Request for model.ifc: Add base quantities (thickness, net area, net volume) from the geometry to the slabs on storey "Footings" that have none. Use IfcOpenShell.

First a look at what the model holds.

```python
import ifcopenshell
import ifcopenshell.util.element
import ifcopenshell.util.unit

model = ifcopenshell.open("model.ifc")
print(model.schema)
for unit_type in ("LENGTHUNIT", "AREAUNIT", "VOLUMEUNIT"):
    print(unit_type, ifcopenshell.util.unit.calculate_unit_scale(model, unit_type))
storey = next(s for s in model.by_type("IfcBuildingStorey") if s.Name == "Footings")
slabs = [e for e in ifcopenshell.util.element.get_decomposition(storey) if e.is_a("IfcSlab")]
for e in sorted(slabs, key=lambda e: e.id()):
    print(e.id(), e.is_a(), e.Name, list(ifcopenshell.util.element.get_psets(e, qtos_only=True)), sep=" | ")
```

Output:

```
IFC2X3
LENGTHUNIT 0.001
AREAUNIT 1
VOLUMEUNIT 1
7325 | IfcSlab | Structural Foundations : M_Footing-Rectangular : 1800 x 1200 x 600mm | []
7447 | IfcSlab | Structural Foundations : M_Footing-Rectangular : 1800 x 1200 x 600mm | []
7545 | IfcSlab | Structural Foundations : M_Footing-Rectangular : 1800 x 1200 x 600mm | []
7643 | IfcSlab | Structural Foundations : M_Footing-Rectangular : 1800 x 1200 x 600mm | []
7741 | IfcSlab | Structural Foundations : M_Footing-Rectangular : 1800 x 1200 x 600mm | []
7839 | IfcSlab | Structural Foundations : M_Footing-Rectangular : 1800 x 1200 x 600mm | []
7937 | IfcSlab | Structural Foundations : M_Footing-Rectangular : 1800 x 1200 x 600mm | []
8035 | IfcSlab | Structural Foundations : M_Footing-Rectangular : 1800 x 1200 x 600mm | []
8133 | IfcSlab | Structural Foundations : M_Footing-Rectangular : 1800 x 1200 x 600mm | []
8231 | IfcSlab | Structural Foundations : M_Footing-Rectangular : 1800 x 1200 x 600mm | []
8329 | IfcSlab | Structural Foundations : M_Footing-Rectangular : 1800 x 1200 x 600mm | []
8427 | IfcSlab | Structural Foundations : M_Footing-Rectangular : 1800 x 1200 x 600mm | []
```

```python
import ifcopenshell
import ifcopenshell.api.pset
import ifcopenshell.geom
import ifcopenshell.util.element
import ifcopenshell.util.shape
import ifcopenshell.util.unit

model = ifcopenshell.open("model.ifc")
unit_scale = ifcopenshell.util.unit.calculate_unit_scale(model)
area_scale = ifcopenshell.util.unit.calculate_unit_scale(model, "AREAUNIT")
volume_scale = ifcopenshell.util.unit.calculate_unit_scale(model, "VOLUMEUNIT")
settings = ifcopenshell.geom.settings()

storey = next(s for s in model.by_type("IfcBuildingStorey") if s.Name == "Footings")
slabs = [e for e in ifcopenshell.util.element.get_decomposition(storey) if e.is_a("IfcSlab")]

for e in sorted(slabs, key=lambda e: e.id()):
    if ifcopenshell.util.element.get_psets(e, qtos_only=True, should_inherit=False):
        continue
    # Geometry comes back in metres, in the element's own axes.
    shape = ifcopenshell.geom.create_shape(settings, e)
    values = {
        "Width": ifcopenshell.util.shape.get_z(shape.geometry) / unit_scale,
        "NetArea": ifcopenshell.util.shape.get_footprint_area(shape.geometry) / area_scale,
        "NetVolume": ifcopenshell.util.shape.get_volume(shape.geometry) / volume_scale,
    }
    qto = ifcopenshell.api.pset.add_qto(model, product=e, name="BaseQuantities")
    ifcopenshell.api.pset.edit_qto(model, qto=qto, properties=values)
    print(e.id(), {k: round(v, 3) for k, v in values.items()})

model.write("model-out.ifc")
```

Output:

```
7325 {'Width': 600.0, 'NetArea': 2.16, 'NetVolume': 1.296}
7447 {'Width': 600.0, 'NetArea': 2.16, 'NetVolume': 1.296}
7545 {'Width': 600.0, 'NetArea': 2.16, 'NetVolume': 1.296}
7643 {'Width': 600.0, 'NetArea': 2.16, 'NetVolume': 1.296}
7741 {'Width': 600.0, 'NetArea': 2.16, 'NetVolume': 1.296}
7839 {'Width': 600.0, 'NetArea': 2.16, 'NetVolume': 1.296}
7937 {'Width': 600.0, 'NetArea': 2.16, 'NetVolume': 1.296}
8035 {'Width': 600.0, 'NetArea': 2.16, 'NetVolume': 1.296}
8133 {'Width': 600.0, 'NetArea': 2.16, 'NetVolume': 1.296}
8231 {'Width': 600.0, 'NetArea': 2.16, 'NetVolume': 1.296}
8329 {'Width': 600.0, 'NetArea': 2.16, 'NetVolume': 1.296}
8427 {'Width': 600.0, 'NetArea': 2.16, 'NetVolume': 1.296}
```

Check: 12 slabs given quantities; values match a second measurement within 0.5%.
